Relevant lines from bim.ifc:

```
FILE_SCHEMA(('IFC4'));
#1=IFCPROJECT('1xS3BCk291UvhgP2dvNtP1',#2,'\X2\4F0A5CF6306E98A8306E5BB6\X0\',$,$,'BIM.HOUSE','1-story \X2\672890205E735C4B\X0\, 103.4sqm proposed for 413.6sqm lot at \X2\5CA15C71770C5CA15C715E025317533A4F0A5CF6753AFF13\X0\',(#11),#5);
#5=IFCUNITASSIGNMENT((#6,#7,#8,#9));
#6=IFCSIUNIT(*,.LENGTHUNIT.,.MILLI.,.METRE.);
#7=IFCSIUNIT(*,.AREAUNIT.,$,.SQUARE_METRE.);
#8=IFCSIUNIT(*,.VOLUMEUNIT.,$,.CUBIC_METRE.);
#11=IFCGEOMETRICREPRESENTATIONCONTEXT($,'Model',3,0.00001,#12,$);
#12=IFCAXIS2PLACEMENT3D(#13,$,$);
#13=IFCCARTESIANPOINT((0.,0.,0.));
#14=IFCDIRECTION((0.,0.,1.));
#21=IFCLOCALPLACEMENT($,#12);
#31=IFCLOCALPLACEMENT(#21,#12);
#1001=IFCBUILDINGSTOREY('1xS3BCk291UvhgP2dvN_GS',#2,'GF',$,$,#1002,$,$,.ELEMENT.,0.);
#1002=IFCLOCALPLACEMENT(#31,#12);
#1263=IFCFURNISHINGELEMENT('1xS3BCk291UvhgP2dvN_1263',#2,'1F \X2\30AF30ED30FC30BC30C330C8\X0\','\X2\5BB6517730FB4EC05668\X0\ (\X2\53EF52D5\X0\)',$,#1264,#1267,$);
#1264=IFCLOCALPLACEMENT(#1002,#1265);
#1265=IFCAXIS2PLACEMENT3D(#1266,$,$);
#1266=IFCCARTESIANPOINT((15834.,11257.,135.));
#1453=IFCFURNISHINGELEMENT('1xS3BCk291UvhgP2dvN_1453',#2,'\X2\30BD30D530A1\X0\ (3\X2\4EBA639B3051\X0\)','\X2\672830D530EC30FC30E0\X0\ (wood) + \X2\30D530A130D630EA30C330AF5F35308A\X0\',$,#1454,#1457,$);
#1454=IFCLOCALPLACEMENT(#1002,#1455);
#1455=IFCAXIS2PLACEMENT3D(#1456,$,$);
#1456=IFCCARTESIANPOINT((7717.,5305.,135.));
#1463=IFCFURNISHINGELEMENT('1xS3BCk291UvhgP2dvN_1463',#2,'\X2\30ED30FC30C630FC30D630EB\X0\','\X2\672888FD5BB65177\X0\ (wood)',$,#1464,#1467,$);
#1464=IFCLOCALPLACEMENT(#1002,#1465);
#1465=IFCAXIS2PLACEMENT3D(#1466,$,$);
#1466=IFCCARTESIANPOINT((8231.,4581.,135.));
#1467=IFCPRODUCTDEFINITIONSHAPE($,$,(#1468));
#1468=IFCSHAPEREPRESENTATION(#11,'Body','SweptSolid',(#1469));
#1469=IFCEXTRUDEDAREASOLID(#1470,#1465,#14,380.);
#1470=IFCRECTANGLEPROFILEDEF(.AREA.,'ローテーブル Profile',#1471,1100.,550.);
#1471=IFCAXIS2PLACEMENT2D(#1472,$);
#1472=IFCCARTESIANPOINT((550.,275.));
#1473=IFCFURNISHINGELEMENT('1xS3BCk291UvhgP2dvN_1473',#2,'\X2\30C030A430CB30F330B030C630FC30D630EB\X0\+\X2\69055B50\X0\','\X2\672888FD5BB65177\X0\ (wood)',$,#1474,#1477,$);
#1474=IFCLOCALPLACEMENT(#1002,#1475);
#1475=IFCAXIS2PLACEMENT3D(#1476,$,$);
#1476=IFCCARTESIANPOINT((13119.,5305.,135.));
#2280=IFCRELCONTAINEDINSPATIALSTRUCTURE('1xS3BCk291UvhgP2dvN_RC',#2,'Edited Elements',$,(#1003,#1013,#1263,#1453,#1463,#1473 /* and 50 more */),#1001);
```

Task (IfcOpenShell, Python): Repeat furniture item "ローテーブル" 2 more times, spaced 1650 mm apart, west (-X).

```python
import numpy as np
import ifcopenshell
import ifcopenshell.api.geometry
import ifcopenshell.api.root
import ifcopenshell.util.element
import ifcopenshell.util.placement
import ifcopenshell.util.unit

model = ifcopenshell.open("bim.ifc")
unit_scale = ifcopenshell.util.unit.calculate_unit_scale(model)


def reuse_history(source, copy):
    """copy_class also copies each property set's owner history, people and application; keep the originals."""
    for rel in copy.IsDefinedBy:
        if rel.is_a("IfcRelDefinesByProperties") and (history := rel.RelatingPropertyDefinition.OwnerHistory):
            rel.RelatingPropertyDefinition.OwnerHistory = source.OwnerHistory
            ifcopenshell.util.element.remove_deep2(model, history)


source = model.by_guid("1xS3BCk291UvhgP2dvN_1463")
base = ifcopenshell.util.placement.get_local_placement(source.ObjectPlacement)
step = np.array([-1.0, 0.0, 0.0]) * 1.65 / unit_scale

for i in range(1, 3):
    copy = ifcopenshell.api.root.copy_class(model, product=source)
    copy.Representation = ifcopenshell.util.element.copy_deep(
        model, source.Representation, exclude=["IfcGeometricRepresentationContext", "IfcRepresentationMap"]
    )
    reuse_history(source, copy)
    matrix = base.copy()
    matrix[:3, 3] += i * step
    print("added at", matrix[:3, 3].round(3) + 0.0)
    ifcopenshell.api.geometry.edit_object_placement(model, product=copy, matrix=matrix, is_si=False)

model.write("bim-out.ifc")
```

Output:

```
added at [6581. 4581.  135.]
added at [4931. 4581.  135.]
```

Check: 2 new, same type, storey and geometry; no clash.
